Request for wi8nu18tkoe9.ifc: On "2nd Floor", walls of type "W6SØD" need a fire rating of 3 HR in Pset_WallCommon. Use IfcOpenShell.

First a look at what the model holds.

```python
import ifcopenshell
import ifcopenshell.util.element

model = ifcopenshell.open("wi8nu18tkoe9.ifc")
print(model.schema)
storey = next(s for s in model.by_type("IfcBuildingStorey") if s.Name == "2nd Floor")
walls = [e for e in ifcopenshell.util.element.get_decomposition(storey) if e.is_a("IfcWall")]
seen = {}
for e in walls:
    element_type = ifcopenshell.util.element.get_type(e)
    key = (element_type.Name if element_type != e and element_type else None, ifcopenshell.util.element.get_pset(e, "Pset_WallCommon", "FireRating"))
    seen[key] = seen.get(key, 0) + 1
for (name, value), count in sorted(seen.items(), key=str):
    print(count, "x", name, "|", value)
```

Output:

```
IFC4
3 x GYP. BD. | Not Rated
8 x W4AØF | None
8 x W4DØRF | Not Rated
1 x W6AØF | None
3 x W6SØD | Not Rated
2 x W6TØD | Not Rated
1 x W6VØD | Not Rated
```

```python
import ifcopenshell
import ifcopenshell.api.pset
import ifcopenshell.util.element

model = ifcopenshell.open("wi8nu18tkoe9.ifc")

storey = next(s for s in model.by_type("IfcBuildingStorey") if s.Name == "2nd Floor")
walls = [e for e in ifcopenshell.util.element.get_decomposition(storey) if e.is_a("IfcWall")]

count = 0
for e in walls:
    element_type = ifcopenshell.util.element.get_type(e)
    if element_type in (None, e) or element_type.Name != "W6SØD":
        continue
    # add_pset returns the element's existing set when there is one.
    pset = ifcopenshell.api.pset.add_pset(model, product=e, name="Pset_WallCommon")
    ifcopenshell.api.pset.edit_pset(model, pset=pset, properties={"FireRating": "3 HR"})
    count += 1

print(count, "walls updated")

model.write("wi8nu18tkoe9-out.ifc")
```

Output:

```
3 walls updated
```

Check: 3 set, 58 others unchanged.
